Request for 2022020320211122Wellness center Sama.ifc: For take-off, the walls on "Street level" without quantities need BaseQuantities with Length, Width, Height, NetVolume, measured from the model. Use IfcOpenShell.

First a look at what the model holds.

```python
import ifcopenshell
import ifcopenshell.util.element
import ifcopenshell.util.unit

model = ifcopenshell.open("2022020320211122Wellness center Sama.ifc")
print(model.schema)
for unit_type in ("LENGTHUNIT", "AREAUNIT", "VOLUMEUNIT"):
    print(unit_type, ifcopenshell.util.unit.calculate_unit_scale(model, unit_type))
storey = next(s for s in model.by_type("IfcBuildingStorey") if s.Name == "Street level")
walls = [e for e in ifcopenshell.util.element.get_decomposition(storey) if e.is_a("IfcWall")]
for e in sorted(walls, key=lambda e: e.id()):
    print(e.id(), e.is_a(), e.Name, list(ifcopenshell.util.element.get_psets(e, qtos_only=True)), sep=" | ")
```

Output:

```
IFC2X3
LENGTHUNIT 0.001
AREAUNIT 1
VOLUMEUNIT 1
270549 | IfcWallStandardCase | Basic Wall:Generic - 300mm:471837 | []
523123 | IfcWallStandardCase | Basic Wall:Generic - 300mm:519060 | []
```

```python
import ifcopenshell
import ifcopenshell.api.pset
import ifcopenshell.geom
import ifcopenshell.util.element
import ifcopenshell.util.shape
import ifcopenshell.util.unit

model = ifcopenshell.open("2022020320211122Wellness center Sama.ifc")
unit_scale = ifcopenshell.util.unit.calculate_unit_scale(model)
volume_scale = ifcopenshell.util.unit.calculate_unit_scale(model, "VOLUMEUNIT")
settings = ifcopenshell.geom.settings()

storey = next(s for s in model.by_type("IfcBuildingStorey") if s.Name == "Street level")
walls = [e for e in ifcopenshell.util.element.get_decomposition(storey) if e.is_a("IfcWall")]

for e in sorted(walls, key=lambda e: e.id()):
    if ifcopenshell.util.element.get_psets(e, qtos_only=True, should_inherit=False):
        continue
    # Geometry comes back in metres, in the element's own axes.
    shape = ifcopenshell.geom.create_shape(settings, e)
    values = {
        "Length": ifcopenshell.util.shape.get_x(shape.geometry) / unit_scale,
        "Width": ifcopenshell.util.shape.get_y(shape.geometry) / unit_scale,
        "Height": ifcopenshell.util.shape.get_z(shape.geometry) / unit_scale,
        "NetVolume": ifcopenshell.util.shape.get_volume(shape.geometry) / volume_scale,
    }
    qto = ifcopenshell.api.pset.add_qto(model, product=e, name="BaseQuantities")
    ifcopenshell.api.pset.edit_qto(model, qto=qto, properties=values)
    print(e.id(), {k: round(v, 3) for k, v in values.items()})

model.write("2022020320211122Wellness center Sama_v2.ifc")
```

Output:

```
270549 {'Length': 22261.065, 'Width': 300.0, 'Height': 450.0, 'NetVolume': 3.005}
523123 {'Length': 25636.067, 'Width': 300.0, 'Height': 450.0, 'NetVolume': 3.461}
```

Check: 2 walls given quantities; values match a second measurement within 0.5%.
